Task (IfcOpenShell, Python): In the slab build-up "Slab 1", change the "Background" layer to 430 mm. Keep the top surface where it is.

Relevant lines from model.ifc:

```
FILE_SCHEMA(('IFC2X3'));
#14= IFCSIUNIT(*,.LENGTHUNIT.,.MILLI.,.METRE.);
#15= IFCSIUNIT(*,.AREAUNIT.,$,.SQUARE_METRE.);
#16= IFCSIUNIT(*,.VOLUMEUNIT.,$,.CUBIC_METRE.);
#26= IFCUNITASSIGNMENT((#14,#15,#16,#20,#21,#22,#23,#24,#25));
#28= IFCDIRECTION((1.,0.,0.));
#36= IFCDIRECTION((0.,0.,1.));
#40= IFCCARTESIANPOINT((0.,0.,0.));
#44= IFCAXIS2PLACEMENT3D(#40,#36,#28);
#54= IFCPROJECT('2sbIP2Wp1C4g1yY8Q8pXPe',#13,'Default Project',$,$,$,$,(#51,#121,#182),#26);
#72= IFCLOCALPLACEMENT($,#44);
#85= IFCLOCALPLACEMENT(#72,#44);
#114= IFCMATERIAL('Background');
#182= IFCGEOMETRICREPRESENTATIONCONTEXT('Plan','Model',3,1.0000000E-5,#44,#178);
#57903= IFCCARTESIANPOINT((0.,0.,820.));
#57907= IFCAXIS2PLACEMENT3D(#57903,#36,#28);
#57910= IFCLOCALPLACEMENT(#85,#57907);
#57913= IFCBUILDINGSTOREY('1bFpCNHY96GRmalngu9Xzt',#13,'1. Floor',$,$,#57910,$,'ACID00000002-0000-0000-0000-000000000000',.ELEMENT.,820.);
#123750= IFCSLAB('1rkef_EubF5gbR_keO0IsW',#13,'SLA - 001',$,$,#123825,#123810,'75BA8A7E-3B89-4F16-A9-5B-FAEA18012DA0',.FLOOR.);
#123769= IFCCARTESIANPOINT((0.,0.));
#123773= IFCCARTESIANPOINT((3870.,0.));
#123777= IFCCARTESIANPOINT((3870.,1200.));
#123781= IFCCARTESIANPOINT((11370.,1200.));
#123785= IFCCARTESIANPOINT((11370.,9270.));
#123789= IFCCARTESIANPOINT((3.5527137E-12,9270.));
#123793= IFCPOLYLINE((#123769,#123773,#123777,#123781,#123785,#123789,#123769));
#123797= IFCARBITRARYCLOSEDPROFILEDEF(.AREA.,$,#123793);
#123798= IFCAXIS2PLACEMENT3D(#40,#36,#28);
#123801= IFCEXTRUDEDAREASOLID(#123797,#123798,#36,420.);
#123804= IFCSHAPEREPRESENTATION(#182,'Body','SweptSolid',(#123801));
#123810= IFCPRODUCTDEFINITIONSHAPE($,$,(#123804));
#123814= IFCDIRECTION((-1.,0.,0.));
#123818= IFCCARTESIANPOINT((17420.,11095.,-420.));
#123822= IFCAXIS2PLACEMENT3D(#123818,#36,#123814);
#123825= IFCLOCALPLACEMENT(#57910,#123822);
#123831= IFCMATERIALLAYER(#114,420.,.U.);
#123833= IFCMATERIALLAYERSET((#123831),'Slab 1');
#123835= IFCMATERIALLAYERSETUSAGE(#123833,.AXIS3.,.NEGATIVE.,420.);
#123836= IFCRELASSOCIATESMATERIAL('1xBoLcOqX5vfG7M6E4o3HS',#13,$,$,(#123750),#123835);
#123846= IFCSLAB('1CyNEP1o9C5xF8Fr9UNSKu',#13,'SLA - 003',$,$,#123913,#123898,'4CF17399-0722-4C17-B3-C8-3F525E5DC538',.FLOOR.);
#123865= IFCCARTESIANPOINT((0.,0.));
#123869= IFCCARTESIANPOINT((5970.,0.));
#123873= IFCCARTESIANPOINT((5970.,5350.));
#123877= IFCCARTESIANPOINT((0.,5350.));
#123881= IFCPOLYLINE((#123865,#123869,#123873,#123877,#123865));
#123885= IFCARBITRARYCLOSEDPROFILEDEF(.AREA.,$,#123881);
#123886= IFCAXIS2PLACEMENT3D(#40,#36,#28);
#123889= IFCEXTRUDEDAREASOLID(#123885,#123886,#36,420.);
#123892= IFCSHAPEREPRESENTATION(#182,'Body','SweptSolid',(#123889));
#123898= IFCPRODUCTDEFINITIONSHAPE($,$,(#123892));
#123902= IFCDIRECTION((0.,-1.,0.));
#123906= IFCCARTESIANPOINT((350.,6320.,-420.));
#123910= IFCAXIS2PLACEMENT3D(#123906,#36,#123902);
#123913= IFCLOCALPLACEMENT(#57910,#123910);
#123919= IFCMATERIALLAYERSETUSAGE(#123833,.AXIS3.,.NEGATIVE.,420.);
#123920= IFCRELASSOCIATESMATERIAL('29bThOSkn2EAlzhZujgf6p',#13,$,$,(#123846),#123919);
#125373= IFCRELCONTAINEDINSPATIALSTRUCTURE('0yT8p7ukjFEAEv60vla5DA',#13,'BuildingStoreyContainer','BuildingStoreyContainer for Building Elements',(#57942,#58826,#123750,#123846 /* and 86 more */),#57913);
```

```python
import ifcopenshell
import ifcopenshell.util.element

model = ifcopenshell.open("model.ifc")

layer_set = model.by_id(123833)
layer = next(l for l in layer_set.MaterialLayers if l.Material and l.Material.Name == "Background")
change = 430.0 - layer.LayerThickness
layer.LayerThickness += change

# The layer set is shared, so every slab that uses it gets the new thickness.
slabs = [e for e in ifcopenshell.util.element.get_elements_by_material(model, layer_set) if e.is_a("IfcSlab")]
for slab in sorted(slabs, key=lambda e: e.id()):
    body = next(r for r in slab.Representation.Representations if r.RepresentationIdentifier == "Body")
    solid = body.Items[0]
    old_depth = solid.Depth
    solid.Depth += change
    # Extruded upwards: lower the start of the extrusion so the top stays.
    x, y, z = solid.Position.Location.Coordinates
    solid.Position.Location = model.createIfcCartesianPoint((x, y, z - change))
    print(slab.id(), f"{old_depth:g} -> {solid.Depth:g}")

model.write("model_rev.ifc")
```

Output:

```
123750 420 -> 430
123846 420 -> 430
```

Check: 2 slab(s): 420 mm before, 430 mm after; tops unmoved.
